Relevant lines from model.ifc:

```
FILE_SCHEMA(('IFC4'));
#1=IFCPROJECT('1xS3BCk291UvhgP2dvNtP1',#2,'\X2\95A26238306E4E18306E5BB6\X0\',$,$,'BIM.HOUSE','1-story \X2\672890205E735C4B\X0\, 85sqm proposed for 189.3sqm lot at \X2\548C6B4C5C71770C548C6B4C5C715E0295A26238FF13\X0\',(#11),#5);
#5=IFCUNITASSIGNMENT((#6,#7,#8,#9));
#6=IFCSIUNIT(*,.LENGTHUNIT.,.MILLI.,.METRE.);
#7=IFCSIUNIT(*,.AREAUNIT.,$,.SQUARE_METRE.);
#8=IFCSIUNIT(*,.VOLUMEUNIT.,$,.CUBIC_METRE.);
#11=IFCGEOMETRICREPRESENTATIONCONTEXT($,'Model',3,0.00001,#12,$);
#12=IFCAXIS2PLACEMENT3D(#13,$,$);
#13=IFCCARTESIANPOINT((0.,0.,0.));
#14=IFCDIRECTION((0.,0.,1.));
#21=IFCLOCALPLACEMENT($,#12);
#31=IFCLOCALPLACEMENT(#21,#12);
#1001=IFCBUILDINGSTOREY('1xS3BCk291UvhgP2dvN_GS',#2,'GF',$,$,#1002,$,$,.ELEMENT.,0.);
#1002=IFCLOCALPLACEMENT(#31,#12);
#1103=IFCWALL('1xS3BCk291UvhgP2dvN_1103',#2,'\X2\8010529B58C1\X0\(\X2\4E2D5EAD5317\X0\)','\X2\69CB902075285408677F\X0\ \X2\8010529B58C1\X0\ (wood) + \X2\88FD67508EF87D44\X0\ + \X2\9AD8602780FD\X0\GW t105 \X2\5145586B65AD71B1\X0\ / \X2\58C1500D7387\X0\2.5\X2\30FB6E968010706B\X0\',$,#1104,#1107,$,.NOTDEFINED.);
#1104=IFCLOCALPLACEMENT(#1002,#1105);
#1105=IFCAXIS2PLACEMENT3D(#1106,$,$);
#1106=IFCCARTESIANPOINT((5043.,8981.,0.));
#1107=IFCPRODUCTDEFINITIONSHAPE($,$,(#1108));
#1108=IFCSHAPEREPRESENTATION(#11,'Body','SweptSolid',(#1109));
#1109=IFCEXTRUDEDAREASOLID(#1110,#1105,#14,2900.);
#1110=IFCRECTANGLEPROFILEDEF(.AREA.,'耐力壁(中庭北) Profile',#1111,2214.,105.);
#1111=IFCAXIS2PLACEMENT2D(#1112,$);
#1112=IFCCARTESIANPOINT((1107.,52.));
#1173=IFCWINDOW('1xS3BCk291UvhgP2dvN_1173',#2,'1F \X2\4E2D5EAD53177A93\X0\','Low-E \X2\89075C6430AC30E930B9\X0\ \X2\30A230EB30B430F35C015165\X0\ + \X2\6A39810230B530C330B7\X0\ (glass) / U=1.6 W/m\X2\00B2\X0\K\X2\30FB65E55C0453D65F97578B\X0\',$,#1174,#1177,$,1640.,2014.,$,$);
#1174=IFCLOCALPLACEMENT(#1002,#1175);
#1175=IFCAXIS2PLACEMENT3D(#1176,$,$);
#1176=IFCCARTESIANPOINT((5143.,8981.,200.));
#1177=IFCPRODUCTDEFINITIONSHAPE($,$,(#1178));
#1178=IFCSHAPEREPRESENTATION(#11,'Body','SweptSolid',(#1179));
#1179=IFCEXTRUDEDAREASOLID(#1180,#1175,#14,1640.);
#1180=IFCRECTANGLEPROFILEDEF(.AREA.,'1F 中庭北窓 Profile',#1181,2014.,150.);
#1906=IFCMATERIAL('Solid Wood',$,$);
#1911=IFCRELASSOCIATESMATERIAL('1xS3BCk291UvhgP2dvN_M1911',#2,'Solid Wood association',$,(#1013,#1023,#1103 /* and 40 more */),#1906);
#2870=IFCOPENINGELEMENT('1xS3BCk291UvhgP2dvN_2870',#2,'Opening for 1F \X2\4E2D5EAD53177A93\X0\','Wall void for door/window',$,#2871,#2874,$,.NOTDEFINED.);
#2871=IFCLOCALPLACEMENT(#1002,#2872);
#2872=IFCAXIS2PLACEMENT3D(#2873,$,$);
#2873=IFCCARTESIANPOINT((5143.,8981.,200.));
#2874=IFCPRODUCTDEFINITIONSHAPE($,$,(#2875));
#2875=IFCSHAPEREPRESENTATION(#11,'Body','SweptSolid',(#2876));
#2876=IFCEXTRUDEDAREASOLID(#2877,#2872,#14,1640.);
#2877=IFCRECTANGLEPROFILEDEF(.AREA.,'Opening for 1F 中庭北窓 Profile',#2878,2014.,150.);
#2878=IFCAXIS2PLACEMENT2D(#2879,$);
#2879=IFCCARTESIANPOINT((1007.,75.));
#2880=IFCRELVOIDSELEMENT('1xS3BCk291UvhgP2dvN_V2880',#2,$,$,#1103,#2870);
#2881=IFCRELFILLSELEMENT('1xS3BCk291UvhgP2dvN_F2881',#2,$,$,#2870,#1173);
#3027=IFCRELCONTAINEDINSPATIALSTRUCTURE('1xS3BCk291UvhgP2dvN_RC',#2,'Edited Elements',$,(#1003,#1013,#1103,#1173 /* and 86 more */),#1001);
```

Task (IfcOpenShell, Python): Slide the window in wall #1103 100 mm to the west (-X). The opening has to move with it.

```python
import ifcopenshell
import ifcopenshell.api.geometry
import ifcopenshell.util.placement

model = ifcopenshell.open("model.ifc")

window = model.by_guid("1xS3BCk291UvhgP2dvN_1173")
opening = window.FillsVoids[0].RelatingOpeningElement
wall = opening.VoidsElements[0].RelatingBuildingElement

wall_matrix = ifcopenshell.util.placement.get_local_placement(wall.ObjectPlacement)
shift = wall_matrix[:3, 0] * -100.0
before = ifcopenshell.util.placement.get_local_placement(window.ObjectPlacement)[:3, 3].copy()

# The window is not placed relative to its opening, so move both.
for product in (opening, window):
    matrix = ifcopenshell.util.placement.get_local_placement(product.ObjectPlacement)
    matrix[:3, 3] += shift
    ifcopenshell.api.geometry.edit_object_placement(model, product=product, matrix=matrix, is_si=False)

after = ifcopenshell.util.placement.get_local_placement(window.ObjectPlacement)[:3, 3]
print("window moved by", (after - before).round(3) + 0.0)

model.write("model_rev.ifc")
```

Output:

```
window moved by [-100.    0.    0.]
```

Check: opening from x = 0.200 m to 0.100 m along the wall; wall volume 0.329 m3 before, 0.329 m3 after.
